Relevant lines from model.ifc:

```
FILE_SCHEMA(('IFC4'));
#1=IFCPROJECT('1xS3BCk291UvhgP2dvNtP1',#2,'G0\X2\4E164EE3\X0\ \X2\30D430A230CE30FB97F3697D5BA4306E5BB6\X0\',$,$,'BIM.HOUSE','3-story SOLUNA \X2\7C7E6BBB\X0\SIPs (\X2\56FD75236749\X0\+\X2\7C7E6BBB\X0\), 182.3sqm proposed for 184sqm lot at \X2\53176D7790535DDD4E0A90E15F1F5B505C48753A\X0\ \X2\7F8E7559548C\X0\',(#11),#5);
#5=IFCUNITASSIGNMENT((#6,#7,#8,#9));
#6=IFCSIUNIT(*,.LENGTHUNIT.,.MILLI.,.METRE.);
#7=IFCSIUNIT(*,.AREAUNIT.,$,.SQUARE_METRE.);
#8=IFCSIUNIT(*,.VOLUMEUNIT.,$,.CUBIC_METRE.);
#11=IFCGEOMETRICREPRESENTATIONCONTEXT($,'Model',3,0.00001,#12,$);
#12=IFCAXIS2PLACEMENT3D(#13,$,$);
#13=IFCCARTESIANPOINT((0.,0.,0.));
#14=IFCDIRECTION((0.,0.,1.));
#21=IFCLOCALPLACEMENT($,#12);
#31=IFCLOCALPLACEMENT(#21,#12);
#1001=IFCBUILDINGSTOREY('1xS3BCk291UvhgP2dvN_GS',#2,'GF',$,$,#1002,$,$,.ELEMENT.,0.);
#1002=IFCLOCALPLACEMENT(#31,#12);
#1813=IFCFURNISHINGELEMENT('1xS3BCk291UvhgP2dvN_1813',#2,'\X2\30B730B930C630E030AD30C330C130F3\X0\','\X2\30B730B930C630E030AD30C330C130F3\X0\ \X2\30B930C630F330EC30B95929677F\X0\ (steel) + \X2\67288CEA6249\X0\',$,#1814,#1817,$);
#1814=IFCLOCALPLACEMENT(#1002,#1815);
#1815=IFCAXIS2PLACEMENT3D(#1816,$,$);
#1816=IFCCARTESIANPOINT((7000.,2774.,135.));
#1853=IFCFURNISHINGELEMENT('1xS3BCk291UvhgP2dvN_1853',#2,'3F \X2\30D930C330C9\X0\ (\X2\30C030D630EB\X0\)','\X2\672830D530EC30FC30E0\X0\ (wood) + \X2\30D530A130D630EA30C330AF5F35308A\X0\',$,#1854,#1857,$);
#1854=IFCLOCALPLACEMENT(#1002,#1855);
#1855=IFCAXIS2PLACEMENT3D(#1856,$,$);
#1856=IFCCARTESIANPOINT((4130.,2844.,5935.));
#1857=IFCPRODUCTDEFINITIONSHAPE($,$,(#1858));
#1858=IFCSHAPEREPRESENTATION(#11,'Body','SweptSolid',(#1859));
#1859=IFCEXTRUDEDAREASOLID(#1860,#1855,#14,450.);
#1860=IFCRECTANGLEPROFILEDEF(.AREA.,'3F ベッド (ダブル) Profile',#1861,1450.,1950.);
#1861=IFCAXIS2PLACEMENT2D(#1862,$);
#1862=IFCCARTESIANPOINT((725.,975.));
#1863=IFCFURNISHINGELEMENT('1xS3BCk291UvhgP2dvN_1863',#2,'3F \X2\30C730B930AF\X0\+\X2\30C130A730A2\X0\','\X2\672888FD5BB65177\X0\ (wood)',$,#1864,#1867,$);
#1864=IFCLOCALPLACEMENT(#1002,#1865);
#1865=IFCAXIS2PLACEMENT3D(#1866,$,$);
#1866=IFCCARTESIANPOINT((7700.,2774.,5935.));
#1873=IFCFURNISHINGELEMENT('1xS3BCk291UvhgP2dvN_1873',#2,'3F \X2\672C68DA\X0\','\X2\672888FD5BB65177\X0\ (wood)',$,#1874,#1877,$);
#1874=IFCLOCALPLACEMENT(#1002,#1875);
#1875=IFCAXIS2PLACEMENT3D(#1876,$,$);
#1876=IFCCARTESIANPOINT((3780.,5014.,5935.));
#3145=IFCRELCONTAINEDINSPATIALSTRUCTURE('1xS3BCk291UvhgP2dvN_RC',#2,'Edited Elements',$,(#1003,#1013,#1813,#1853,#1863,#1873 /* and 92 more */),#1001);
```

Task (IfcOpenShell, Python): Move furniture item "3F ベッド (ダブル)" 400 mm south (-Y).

```python
import ifcopenshell
import ifcopenshell.api.geometry
import ifcopenshell.util.placement
import ifcopenshell.util.unit

model = ifcopenshell.open("model.ifc")
unit_scale = ifcopenshell.util.unit.calculate_unit_scale(model)

item = model.by_guid("1xS3BCk291UvhgP2dvN_1853")
matrix = ifcopenshell.util.placement.get_local_placement(item.ObjectPlacement)
matrix[1, 3] -= 0.4 / unit_scale
ifcopenshell.api.geometry.edit_object_placement(model, product=item, matrix=matrix, is_si=False)

print(ifcopenshell.util.placement.get_local_placement(item.ObjectPlacement).round(3) + 0.0)

model.write("model_rev.ifc")
```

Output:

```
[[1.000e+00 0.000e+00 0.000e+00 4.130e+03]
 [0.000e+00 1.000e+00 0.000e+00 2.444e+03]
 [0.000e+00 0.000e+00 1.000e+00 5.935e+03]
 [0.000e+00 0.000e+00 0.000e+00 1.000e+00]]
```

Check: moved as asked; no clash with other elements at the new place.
